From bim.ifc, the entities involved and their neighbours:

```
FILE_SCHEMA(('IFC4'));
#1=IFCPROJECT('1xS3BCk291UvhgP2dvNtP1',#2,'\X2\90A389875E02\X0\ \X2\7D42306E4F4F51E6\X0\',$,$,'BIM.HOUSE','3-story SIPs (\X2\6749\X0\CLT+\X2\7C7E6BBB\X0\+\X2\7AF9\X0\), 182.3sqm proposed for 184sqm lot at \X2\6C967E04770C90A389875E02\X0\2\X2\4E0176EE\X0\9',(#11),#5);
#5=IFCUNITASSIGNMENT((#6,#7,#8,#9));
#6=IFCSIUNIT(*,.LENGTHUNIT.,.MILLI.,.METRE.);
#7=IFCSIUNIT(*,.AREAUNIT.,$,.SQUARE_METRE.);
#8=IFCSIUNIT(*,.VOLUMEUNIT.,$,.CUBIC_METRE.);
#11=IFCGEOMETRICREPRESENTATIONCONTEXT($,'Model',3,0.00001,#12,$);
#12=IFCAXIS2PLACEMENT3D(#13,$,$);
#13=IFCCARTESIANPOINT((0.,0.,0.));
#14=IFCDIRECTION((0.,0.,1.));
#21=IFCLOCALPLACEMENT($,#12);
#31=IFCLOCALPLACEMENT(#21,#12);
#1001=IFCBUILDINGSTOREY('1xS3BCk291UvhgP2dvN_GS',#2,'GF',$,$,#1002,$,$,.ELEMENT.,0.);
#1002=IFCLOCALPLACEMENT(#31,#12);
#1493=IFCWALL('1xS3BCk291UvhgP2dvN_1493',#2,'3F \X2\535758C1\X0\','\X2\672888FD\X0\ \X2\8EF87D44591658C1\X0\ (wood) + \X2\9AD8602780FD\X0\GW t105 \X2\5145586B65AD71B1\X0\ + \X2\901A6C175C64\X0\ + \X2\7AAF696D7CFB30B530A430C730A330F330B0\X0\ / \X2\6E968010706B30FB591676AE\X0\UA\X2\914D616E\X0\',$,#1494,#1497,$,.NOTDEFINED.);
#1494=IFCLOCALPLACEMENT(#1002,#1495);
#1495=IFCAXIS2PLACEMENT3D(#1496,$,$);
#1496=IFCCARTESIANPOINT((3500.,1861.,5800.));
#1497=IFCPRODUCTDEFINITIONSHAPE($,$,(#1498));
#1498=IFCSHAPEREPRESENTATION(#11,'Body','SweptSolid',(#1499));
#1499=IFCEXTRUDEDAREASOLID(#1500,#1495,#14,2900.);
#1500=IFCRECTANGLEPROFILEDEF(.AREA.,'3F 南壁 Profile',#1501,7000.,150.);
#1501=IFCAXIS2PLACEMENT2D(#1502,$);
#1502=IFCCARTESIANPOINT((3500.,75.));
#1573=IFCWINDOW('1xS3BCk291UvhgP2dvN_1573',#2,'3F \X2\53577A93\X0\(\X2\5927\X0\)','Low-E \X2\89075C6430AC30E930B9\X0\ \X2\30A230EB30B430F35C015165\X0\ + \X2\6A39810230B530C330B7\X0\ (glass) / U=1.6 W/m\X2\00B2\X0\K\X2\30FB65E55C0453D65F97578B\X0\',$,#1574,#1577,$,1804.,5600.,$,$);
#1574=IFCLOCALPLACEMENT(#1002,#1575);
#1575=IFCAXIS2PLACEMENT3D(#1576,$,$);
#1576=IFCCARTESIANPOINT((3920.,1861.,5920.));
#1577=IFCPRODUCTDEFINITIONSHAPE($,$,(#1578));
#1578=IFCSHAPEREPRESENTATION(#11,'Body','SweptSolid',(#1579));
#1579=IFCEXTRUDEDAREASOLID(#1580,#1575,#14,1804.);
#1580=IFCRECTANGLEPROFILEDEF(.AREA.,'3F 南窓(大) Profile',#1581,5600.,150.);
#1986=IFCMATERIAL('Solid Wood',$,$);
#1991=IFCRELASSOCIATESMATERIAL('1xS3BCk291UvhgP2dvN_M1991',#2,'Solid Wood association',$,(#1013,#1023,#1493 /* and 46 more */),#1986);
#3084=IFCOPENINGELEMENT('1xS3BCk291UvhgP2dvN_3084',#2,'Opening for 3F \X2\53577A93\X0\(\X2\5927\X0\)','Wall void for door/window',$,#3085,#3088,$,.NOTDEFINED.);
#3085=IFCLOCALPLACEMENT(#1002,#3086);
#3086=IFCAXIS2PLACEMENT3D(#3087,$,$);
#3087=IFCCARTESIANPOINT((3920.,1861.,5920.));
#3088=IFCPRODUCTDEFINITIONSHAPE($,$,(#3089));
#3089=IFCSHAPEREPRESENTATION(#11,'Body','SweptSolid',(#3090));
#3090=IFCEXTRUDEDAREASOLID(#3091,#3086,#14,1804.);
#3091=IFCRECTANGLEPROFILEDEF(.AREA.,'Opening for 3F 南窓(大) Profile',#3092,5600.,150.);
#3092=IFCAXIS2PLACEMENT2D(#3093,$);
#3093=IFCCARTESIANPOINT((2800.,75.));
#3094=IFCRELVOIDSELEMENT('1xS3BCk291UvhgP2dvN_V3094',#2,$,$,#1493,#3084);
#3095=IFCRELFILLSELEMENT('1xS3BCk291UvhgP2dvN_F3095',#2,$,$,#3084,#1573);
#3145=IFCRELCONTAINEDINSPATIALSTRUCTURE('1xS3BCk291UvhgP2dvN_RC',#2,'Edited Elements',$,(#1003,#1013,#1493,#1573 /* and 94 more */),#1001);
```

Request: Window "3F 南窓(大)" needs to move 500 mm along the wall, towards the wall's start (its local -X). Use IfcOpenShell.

```python
import ifcopenshell
import ifcopenshell.api.geometry
import ifcopenshell.util.placement

model = ifcopenshell.open("bim.ifc")

window = model.by_guid("1xS3BCk291UvhgP2dvN_1573")
opening = window.FillsVoids[0].RelatingOpeningElement
wall = opening.VoidsElements[0].RelatingBuildingElement

wall_matrix = ifcopenshell.util.placement.get_local_placement(wall.ObjectPlacement)
shift = wall_matrix[:3, 0] * -500.0
before = ifcopenshell.util.placement.get_local_placement(window.ObjectPlacement)[:3, 3].copy()

# The window is not placed relative to its opening, so move both.
for product in (opening, window):
    matrix = ifcopenshell.util.placement.get_local_placement(product.ObjectPlacement)
    matrix[:3, 3] += shift
    ifcopenshell.api.geometry.edit_object_placement(model, product=product, matrix=matrix, is_si=False)

after = ifcopenshell.util.placement.get_local_placement(window.ObjectPlacement)[:3, 3]
print("window moved by", (after - before).round(3) + 0.0)

model.write("bim_v2.ifc")
```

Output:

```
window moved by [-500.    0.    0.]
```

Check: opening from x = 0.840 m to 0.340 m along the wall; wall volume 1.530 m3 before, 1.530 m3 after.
